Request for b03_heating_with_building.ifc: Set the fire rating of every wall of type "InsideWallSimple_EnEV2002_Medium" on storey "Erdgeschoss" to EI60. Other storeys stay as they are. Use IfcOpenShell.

First a look at what the model holds.

```python
import ifcopenshell
import ifcopenshell.util.element

model = ifcopenshell.open("b03_heating_with_building.ifc")
print(model.schema)
storey = next(s for s in model.by_type("IfcBuildingStorey") if s.Name == "Erdgeschoss")
walls = [e for e in ifcopenshell.util.element.get_decomposition(storey) if e.is_a("IfcWall")]
seen = {}
for e in walls:
    element_type = ifcopenshell.util.element.get_type(e)
    key = (element_type.Name if element_type != e and element_type else None, ifcopenshell.util.element.get_pset(e, "Pset_WallCommon", "FireRating"))
    seen[key] = seen.get(key, 0) + 1
for (name, value), count in sorted(seen.items(), key=str):
    print(count, "x", name, "|", value)
```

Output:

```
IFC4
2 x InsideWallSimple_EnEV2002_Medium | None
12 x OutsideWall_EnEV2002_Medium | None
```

```python
import ifcopenshell
import ifcopenshell.api.pset
import ifcopenshell.util.element

model = ifcopenshell.open("b03_heating_with_building.ifc")

storey = next(s for s in model.by_type("IfcBuildingStorey") if s.Name == "Erdgeschoss")
walls = [e for e in ifcopenshell.util.element.get_decomposition(storey) if e.is_a("IfcWall")]

count = 0
for e in walls:
    element_type = ifcopenshell.util.element.get_type(e)
    if element_type in (None, e) or element_type.Name != "InsideWallSimple_EnEV2002_Medium":
        continue
    # add_pset returns the element's existing set when there is one.
    pset = ifcopenshell.api.pset.add_pset(model, product=e, name="Pset_WallCommon")
    ifcopenshell.api.pset.edit_pset(model, pset=pset, properties={"FireRating": "EI60"})
    count += 1

print(count, "walls updated")

model.write("b03_heating_with_building-out.ifc")
```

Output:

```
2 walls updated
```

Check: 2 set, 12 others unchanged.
